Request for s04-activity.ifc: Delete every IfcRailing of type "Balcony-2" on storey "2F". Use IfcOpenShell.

First a look at what the model holds.

```python
import ifcopenshell
import ifcopenshell.util.element

model = ifcopenshell.open("s04-activity.ifc")
print(model.schema)
storey = next(s for s in model.by_type("IfcBuildingStorey") if s.Name == "2F")
railings = [e for e in ifcopenshell.util.element.get_decomposition(storey) if e.is_a("IfcRailing")]
seen = {}
for e in railings:
    element_type = ifcopenshell.util.element.get_type(e)
    name = element_type.Name if element_type not in (None, e) else None
    seen[name] = seen.get(name, 0) + 1
for name, count in sorted(seen.items(), key=str):
    print(count, "x", name)
```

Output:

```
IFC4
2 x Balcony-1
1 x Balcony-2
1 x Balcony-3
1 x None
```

```python
import ifcopenshell
import ifcopenshell.api.root
import ifcopenshell.util.element

model = ifcopenshell.open("s04-activity.ifc")

storey = next(s for s in model.by_type("IfcBuildingStorey") if s.Name == "2F")
railings = [e for e in ifcopenshell.util.element.get_decomposition(storey) if e.is_a("IfcRailing")]
targets = [e for e in railings if (t := ifcopenshell.util.element.get_type(e)) not in (None, e) and t.Name == "Balcony-2"]

for e in targets:
    ifcopenshell.api.root.remove_product(model, product=e)
print(len(targets), "removed")

model.write("s04-activity_edited.ifc")
```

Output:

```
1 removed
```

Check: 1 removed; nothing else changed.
